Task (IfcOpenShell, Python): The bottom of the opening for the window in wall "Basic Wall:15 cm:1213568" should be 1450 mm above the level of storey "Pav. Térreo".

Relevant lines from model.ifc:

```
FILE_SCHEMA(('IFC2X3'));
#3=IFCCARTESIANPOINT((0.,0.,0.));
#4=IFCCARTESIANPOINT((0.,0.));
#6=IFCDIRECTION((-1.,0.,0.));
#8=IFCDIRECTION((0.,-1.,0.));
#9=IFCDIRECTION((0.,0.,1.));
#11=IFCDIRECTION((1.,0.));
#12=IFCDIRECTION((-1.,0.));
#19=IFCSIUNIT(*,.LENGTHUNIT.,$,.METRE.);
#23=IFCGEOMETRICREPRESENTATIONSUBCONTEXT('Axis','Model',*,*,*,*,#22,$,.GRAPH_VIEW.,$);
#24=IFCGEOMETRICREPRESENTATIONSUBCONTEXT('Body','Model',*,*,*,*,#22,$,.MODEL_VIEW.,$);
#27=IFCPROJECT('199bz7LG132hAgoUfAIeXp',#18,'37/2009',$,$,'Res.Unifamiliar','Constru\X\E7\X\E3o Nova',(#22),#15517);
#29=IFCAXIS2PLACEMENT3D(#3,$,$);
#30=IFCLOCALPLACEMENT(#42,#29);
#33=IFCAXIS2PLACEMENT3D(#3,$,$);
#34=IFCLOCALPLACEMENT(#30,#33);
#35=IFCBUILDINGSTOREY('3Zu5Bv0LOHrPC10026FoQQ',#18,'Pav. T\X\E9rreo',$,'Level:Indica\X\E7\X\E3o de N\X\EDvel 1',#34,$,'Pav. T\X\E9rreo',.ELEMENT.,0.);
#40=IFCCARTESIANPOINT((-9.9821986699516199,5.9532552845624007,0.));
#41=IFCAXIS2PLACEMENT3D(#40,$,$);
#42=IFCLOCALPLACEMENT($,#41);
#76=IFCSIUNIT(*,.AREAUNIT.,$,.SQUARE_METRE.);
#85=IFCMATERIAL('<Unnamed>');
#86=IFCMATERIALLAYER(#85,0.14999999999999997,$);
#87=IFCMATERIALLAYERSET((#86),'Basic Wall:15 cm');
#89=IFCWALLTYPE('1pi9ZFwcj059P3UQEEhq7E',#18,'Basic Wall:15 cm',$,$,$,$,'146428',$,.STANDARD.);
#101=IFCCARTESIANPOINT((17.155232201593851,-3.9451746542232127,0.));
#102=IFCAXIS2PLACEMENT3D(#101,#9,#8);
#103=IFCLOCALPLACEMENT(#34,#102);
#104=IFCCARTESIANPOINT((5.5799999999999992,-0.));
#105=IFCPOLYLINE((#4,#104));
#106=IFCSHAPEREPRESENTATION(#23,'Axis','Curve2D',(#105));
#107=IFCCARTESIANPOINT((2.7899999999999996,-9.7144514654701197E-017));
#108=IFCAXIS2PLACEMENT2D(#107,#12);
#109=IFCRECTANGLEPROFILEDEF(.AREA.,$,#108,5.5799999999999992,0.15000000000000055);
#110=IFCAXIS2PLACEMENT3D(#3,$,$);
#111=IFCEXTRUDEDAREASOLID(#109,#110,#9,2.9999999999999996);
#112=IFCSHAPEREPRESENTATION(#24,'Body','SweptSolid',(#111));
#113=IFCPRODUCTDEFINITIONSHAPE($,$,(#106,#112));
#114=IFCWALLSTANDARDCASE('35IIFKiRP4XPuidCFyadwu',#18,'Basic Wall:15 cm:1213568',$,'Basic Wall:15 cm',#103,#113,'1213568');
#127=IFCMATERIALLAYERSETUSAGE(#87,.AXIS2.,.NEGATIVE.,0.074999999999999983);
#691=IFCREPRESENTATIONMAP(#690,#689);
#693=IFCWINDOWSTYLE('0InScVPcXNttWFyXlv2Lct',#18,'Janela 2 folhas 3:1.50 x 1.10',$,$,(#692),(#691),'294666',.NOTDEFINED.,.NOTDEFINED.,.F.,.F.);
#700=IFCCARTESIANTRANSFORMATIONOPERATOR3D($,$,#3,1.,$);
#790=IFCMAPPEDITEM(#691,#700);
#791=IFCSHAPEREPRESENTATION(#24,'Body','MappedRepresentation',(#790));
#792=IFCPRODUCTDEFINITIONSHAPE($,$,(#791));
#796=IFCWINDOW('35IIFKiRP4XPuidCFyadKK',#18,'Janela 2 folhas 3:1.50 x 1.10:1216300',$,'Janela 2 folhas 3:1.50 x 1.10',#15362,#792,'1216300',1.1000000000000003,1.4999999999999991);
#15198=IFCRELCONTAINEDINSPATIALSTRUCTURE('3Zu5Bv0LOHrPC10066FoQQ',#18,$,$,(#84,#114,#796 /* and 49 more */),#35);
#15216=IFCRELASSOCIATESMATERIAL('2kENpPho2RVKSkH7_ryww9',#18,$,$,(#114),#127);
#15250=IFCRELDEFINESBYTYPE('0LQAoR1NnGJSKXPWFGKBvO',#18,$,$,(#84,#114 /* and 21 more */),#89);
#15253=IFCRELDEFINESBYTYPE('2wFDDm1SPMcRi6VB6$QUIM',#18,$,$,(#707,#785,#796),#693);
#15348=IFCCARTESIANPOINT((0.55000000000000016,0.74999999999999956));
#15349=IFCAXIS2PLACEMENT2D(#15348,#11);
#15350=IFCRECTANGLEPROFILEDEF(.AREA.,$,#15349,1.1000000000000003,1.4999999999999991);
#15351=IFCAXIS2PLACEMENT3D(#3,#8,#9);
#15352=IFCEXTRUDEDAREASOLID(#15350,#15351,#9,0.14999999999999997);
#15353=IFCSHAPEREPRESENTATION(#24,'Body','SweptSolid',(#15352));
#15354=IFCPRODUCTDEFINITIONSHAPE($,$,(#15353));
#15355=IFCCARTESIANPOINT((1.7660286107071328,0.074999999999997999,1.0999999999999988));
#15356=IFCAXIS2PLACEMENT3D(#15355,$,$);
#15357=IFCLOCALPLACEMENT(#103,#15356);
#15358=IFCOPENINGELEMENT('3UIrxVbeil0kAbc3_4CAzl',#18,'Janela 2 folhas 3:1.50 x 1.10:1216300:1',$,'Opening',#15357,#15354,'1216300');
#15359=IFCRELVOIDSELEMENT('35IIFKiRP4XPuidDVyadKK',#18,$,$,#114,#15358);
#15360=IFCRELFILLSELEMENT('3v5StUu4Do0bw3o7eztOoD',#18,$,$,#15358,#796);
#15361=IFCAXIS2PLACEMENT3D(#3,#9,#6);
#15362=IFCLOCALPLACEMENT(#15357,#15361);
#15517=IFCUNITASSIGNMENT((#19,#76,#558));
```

```python
import numpy as np
import ifcopenshell
import ifcopenshell.api.geometry
import ifcopenshell.geom
import ifcopenshell.util.element
import ifcopenshell.util.placement
import ifcopenshell.util.shape
import ifcopenshell.util.unit

model = ifcopenshell.open("model.ifc")
unit_scale = ifcopenshell.util.unit.calculate_unit_scale(model)

window = model.by_guid("35IIFKiRP4XPuidCFyadKK")
opening = window.FillsVoids[0].RelatingOpeningElement
storey = ifcopenshell.util.element.get_container(window, ifc_class="IfcBuildingStorey")
level = ifcopenshell.util.placement.get_local_placement(storey.ObjectPlacement)[2, 3]

# The opening's origin need not be at the sill, so measure its lowest point.
shape = ifcopenshell.geom.create_shape(ifcopenshell.geom.settings(), opening)
bottom = ifcopenshell.util.shape.get_shape_bottom_elevation(shape, shape.geometry) / unit_scale
dz = level + 1.45 - bottom

shift = np.array([0.0, 0.0, dz])
# The window is placed relative to its opening, so it follows when the opening moves.
matrix = ifcopenshell.util.placement.get_local_placement(opening.ObjectPlacement)
matrix[:3, 3] += shift
ifcopenshell.api.geometry.edit_object_placement(
    model, product=opening, matrix=matrix, is_si=False, should_transform_children=True
)

print(f"moved by {dz * unit_scale:+.3f} m")

model.write("model_updated.ifc")
```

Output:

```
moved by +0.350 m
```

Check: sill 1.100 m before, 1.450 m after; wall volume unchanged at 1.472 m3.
